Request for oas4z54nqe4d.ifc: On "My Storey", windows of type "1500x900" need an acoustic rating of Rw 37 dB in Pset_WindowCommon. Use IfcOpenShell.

First a look at what the model holds.

```python
import ifcopenshell
import ifcopenshell.util.element

model = ifcopenshell.open("oas4z54nqe4d.ifc")
print(model.schema)
storey = next(s for s in model.by_type("IfcBuildingStorey") if s.Name == "My Storey")
windows = [e for e in ifcopenshell.util.element.get_decomposition(storey) if e.is_a("IfcWindow")]
seen = {}
for e in windows:
    element_type = ifcopenshell.util.element.get_type(e)
    key = (element_type.Name if element_type != e and element_type else None, ifcopenshell.util.element.get_pset(e, "Pset_WindowCommon", "AcousticRating"))
    seen[key] = seen.get(key, 0) + 1
for (name, value), count in sorted(seen.items(), key=str):
    print(count, "x", name, "|", value)
```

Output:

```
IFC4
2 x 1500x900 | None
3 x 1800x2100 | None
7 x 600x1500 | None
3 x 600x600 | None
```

```python
import ifcopenshell
import ifcopenshell.api.pset
import ifcopenshell.util.element

model = ifcopenshell.open("oas4z54nqe4d.ifc")

storey = next(s for s in model.by_type("IfcBuildingStorey") if s.Name == "My Storey")
windows = [e for e in ifcopenshell.util.element.get_decomposition(storey) if e.is_a("IfcWindow")]

count = 0
for e in windows:
    element_type = ifcopenshell.util.element.get_type(e)
    if element_type in (None, e) or element_type.Name != "1500x900":
        continue
    # add_pset returns the element's existing set when there is one.
    pset = ifcopenshell.api.pset.add_pset(model, product=e, name="Pset_WindowCommon")
    ifcopenshell.api.pset.edit_pset(model, pset=pset, properties={"AcousticRating": "Rw 37 dB"})
    count += 1

print(count, "windows updated")

model.write("oas4z54nqe4d_rev.ifc")
```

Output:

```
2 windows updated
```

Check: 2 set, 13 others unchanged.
